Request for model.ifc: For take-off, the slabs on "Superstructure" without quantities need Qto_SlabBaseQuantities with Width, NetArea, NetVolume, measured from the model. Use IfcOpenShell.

First a look at what the model holds.

```python
import ifcopenshell
import ifcopenshell.util.element
import ifcopenshell.util.unit

model = ifcopenshell.open("model.ifc")
print(model.schema)
for unit_type in ("LENGTHUNIT", "AREAUNIT", "VOLUMEUNIT"):
    print(unit_type, ifcopenshell.util.unit.calculate_unit_scale(model, unit_type))
storey = next(s for s in model.by_type("IfcBuildingStorey") if s.Name == "Superstructure")
slabs = [e for e in ifcopenshell.util.element.get_decomposition(storey) if e.is_a("IfcSlab")]
for e in sorted(slabs, key=lambda e: e.id()):
    print(e.id(), e.is_a(), e.Name, list(ifcopenshell.util.element.get_psets(e, qtos_only=True)), sep=" | ")
```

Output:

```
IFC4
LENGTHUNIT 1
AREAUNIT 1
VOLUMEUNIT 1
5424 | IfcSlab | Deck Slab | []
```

```python
import ifcopenshell
import ifcopenshell.api.pset
import ifcopenshell.geom
import ifcopenshell.util.element
import ifcopenshell.util.shape
import ifcopenshell.util.unit

model = ifcopenshell.open("model.ifc")
unit_scale = ifcopenshell.util.unit.calculate_unit_scale(model)
area_scale = ifcopenshell.util.unit.calculate_unit_scale(model, "AREAUNIT")
volume_scale = ifcopenshell.util.unit.calculate_unit_scale(model, "VOLUMEUNIT")
settings = ifcopenshell.geom.settings()

storey = next(s for s in model.by_type("IfcBuildingStorey") if s.Name == "Superstructure")
slabs = [e for e in ifcopenshell.util.element.get_decomposition(storey) if e.is_a("IfcSlab")]

for e in sorted(slabs, key=lambda e: e.id()):
    if ifcopenshell.util.element.get_psets(e, qtos_only=True, should_inherit=False):
        continue
    # Geometry comes back in metres, in the element's own axes.
    shape = ifcopenshell.geom.create_shape(settings, e)
    values = {
        "Width": ifcopenshell.util.shape.get_z(shape.geometry) / unit_scale,
        "NetArea": ifcopenshell.util.shape.get_footprint_area(shape.geometry) / area_scale,
        "NetVolume": ifcopenshell.util.shape.get_volume(shape.geometry) / volume_scale,
    }
    qto = ifcopenshell.api.pset.add_qto(model, product=e, name="Qto_SlabBaseQuantities")
    ifcopenshell.api.pset.edit_qto(model, qto=qto, properties=values)
    print(e.id(), {k: round(v, 3) for k, v in values.items()})

model.write("model_v2.ifc")
```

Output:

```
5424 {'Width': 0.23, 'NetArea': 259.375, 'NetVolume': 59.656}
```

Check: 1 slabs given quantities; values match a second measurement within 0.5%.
